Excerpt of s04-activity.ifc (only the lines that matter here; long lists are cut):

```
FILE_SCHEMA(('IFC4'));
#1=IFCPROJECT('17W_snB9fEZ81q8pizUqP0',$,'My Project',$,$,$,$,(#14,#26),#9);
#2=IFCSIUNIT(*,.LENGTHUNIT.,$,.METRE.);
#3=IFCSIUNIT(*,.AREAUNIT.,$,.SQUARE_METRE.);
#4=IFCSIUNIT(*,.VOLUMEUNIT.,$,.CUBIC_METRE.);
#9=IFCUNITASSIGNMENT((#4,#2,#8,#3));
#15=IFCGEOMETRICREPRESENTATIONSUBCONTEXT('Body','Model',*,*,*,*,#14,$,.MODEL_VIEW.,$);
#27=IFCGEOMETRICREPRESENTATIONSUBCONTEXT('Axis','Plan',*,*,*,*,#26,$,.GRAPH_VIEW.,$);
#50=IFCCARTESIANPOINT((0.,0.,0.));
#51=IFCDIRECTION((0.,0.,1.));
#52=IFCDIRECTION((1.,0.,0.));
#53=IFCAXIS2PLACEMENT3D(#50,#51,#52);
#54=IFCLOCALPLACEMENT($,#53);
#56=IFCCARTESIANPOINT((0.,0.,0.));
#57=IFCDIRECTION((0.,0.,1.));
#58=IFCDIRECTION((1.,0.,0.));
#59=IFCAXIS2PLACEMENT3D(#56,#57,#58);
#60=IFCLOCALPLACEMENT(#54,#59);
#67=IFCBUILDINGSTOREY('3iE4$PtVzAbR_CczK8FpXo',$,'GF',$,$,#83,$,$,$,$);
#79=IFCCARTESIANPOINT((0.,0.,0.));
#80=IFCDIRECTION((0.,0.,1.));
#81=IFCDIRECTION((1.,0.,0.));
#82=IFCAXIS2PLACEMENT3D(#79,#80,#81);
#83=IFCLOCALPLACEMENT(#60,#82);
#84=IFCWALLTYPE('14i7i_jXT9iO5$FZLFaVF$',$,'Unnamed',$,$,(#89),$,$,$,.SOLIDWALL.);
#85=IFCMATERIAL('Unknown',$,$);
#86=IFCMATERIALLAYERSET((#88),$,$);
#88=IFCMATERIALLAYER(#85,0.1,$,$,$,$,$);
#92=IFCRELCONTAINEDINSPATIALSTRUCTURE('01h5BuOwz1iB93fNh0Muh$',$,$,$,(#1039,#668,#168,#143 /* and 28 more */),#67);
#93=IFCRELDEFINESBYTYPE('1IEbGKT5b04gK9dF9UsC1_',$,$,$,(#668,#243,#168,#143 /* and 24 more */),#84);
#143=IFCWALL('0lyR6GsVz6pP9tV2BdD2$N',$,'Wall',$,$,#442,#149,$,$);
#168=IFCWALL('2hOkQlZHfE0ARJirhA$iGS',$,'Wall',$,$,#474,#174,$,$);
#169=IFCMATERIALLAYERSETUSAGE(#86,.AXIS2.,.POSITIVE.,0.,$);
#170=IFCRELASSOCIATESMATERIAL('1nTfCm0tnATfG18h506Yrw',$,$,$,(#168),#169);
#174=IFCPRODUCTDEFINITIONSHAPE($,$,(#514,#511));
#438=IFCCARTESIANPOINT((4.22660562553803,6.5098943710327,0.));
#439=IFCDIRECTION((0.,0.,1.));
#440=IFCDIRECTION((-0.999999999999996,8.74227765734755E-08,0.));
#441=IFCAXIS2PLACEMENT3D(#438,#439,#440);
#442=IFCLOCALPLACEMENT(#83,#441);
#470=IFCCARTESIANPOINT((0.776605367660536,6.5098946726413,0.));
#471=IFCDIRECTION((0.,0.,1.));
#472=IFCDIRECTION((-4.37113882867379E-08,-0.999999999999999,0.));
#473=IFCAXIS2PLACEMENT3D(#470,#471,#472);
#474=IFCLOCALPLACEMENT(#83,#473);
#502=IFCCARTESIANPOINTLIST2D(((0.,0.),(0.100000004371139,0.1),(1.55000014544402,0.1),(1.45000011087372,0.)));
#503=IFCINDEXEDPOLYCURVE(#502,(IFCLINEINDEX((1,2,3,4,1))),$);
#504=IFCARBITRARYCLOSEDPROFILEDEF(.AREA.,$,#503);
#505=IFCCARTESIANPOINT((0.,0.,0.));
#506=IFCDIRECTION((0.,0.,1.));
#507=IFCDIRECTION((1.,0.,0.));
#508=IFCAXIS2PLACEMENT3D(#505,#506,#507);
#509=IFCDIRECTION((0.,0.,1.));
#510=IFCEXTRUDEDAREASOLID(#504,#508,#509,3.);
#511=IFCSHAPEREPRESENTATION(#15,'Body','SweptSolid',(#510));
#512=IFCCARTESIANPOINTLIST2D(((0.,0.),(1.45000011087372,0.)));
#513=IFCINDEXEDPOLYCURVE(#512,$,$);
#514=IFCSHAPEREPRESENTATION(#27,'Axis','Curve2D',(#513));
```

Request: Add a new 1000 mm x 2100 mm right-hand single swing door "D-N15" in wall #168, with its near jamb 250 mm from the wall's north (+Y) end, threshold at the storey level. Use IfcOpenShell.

```python
import numpy as np
import ifcopenshell
import ifcopenshell.api.feature
import ifcopenshell.api.geometry
import ifcopenshell.api.root
import ifcopenshell.api.spatial
import ifcopenshell.geom
import ifcopenshell.util.element
import ifcopenshell.util.placement
import ifcopenshell.util.representation
import ifcopenshell.util.shape
import ifcopenshell.util.unit

model = ifcopenshell.open("s04-activity.ifc")
unit_scale = ifcopenshell.util.unit.calculate_unit_scale(model)
settings = ifcopenshell.geom.settings()


def volume(element):
    """Net volume in cubic metres, openings subtracted."""
    shape = ifcopenshell.geom.create_shape(settings, element)
    return ifcopenshell.util.shape.get_volume(shape.geometry)


wall = model.by_guid("2hOkQlZHfE0ARJirhA$iGS")
storey = ifcopenshell.util.element.get_container(wall, ifc_class="IfcBuildingStorey")
context = ifcopenshell.util.representation.get_context(model, "Model", "Body", "MODEL_VIEW")
before = volume(wall)

width, height, from_end, sill = 1, 2.1, 0.25, 0.0  # metres

# The wall runs along its own X axis, and the end named is its -X end.
wall_shape = ifcopenshell.geom.create_shape(settings, wall)
x, y, z = ifcopenshell.util.shape.get_vertices(wall_shape.geometry).T
start = x.min() + from_end
face, thickness = float(y.min()), float(y.max() - y.min())
wall_matrix = ifcopenshell.util.placement.get_local_placement(wall.ObjectPlacement)
level = ifcopenshell.util.placement.get_local_placement(storey.ObjectPlacement)[2, 3]


def in_wall(x, y):
    """Placement at x, y metres in the wall's axes, at sill height."""
    matrix = wall_matrix.copy()
    matrix[:, 3] = wall_matrix @ np.array([x / unit_scale, y / unit_scale, 0.0, 1.0])
    matrix[2, 3] = level + sill / unit_scale
    return matrix


# Opening: a box that overshoots both wall faces by 50 mm.
opening = ifcopenshell.api.root.create_entity(model, ifc_class="IfcOpeningElement", predefined_type="OPENING")
box = ifcopenshell.api.geometry.add_wall_representation(
    model, context=context, length=width, height=height, thickness=thickness + 0.1
)
ifcopenshell.api.geometry.assign_representation(model, product=opening, representation=box)
ifcopenshell.api.geometry.edit_object_placement(model, product=opening, matrix=in_wall(start, face - 0.05), is_si=False)
ifcopenshell.api.feature.add_feature(model, feature=opening, element=wall)

door = ifcopenshell.api.root.create_entity(model, ifc_class="IfcDoor", name="D-N15", predefined_type="DOOR")
door.OverallWidth, door.OverallHeight = width / unit_scale, height / unit_scale
door.OperationType = "SINGLE_SWING_RIGHT"
body = ifcopenshell.api.geometry.add_door_representation(
    model,
    context=context,
    overall_width=door.OverallWidth,
    overall_height=door.OverallHeight,
    operation_type="SINGLE_SWING_RIGHT",
    lining_properties={"LiningDepth": thickness / unit_scale, "ThresholdDepth": thickness / unit_scale},
)
ifcopenshell.api.geometry.assign_representation(model, product=door, representation=body)
ifcopenshell.api.spatial.assign_container(model, products=[door], relating_structure=storey)
ifcopenshell.api.feature.add_filling(model, opening=opening, element=door)

# The lining spans the wall, so the door starts at the wall face.
ifcopenshell.api.geometry.edit_object_placement(model, product=door, matrix=in_wall(start, face), is_si=False)

after = volume(wall)

print(f"wall volume {before:.3f} -> {after:.3f} m3")

model.write("s04-activity_v2.ifc")
```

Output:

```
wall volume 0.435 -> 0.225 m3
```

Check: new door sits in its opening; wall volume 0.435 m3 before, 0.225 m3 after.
